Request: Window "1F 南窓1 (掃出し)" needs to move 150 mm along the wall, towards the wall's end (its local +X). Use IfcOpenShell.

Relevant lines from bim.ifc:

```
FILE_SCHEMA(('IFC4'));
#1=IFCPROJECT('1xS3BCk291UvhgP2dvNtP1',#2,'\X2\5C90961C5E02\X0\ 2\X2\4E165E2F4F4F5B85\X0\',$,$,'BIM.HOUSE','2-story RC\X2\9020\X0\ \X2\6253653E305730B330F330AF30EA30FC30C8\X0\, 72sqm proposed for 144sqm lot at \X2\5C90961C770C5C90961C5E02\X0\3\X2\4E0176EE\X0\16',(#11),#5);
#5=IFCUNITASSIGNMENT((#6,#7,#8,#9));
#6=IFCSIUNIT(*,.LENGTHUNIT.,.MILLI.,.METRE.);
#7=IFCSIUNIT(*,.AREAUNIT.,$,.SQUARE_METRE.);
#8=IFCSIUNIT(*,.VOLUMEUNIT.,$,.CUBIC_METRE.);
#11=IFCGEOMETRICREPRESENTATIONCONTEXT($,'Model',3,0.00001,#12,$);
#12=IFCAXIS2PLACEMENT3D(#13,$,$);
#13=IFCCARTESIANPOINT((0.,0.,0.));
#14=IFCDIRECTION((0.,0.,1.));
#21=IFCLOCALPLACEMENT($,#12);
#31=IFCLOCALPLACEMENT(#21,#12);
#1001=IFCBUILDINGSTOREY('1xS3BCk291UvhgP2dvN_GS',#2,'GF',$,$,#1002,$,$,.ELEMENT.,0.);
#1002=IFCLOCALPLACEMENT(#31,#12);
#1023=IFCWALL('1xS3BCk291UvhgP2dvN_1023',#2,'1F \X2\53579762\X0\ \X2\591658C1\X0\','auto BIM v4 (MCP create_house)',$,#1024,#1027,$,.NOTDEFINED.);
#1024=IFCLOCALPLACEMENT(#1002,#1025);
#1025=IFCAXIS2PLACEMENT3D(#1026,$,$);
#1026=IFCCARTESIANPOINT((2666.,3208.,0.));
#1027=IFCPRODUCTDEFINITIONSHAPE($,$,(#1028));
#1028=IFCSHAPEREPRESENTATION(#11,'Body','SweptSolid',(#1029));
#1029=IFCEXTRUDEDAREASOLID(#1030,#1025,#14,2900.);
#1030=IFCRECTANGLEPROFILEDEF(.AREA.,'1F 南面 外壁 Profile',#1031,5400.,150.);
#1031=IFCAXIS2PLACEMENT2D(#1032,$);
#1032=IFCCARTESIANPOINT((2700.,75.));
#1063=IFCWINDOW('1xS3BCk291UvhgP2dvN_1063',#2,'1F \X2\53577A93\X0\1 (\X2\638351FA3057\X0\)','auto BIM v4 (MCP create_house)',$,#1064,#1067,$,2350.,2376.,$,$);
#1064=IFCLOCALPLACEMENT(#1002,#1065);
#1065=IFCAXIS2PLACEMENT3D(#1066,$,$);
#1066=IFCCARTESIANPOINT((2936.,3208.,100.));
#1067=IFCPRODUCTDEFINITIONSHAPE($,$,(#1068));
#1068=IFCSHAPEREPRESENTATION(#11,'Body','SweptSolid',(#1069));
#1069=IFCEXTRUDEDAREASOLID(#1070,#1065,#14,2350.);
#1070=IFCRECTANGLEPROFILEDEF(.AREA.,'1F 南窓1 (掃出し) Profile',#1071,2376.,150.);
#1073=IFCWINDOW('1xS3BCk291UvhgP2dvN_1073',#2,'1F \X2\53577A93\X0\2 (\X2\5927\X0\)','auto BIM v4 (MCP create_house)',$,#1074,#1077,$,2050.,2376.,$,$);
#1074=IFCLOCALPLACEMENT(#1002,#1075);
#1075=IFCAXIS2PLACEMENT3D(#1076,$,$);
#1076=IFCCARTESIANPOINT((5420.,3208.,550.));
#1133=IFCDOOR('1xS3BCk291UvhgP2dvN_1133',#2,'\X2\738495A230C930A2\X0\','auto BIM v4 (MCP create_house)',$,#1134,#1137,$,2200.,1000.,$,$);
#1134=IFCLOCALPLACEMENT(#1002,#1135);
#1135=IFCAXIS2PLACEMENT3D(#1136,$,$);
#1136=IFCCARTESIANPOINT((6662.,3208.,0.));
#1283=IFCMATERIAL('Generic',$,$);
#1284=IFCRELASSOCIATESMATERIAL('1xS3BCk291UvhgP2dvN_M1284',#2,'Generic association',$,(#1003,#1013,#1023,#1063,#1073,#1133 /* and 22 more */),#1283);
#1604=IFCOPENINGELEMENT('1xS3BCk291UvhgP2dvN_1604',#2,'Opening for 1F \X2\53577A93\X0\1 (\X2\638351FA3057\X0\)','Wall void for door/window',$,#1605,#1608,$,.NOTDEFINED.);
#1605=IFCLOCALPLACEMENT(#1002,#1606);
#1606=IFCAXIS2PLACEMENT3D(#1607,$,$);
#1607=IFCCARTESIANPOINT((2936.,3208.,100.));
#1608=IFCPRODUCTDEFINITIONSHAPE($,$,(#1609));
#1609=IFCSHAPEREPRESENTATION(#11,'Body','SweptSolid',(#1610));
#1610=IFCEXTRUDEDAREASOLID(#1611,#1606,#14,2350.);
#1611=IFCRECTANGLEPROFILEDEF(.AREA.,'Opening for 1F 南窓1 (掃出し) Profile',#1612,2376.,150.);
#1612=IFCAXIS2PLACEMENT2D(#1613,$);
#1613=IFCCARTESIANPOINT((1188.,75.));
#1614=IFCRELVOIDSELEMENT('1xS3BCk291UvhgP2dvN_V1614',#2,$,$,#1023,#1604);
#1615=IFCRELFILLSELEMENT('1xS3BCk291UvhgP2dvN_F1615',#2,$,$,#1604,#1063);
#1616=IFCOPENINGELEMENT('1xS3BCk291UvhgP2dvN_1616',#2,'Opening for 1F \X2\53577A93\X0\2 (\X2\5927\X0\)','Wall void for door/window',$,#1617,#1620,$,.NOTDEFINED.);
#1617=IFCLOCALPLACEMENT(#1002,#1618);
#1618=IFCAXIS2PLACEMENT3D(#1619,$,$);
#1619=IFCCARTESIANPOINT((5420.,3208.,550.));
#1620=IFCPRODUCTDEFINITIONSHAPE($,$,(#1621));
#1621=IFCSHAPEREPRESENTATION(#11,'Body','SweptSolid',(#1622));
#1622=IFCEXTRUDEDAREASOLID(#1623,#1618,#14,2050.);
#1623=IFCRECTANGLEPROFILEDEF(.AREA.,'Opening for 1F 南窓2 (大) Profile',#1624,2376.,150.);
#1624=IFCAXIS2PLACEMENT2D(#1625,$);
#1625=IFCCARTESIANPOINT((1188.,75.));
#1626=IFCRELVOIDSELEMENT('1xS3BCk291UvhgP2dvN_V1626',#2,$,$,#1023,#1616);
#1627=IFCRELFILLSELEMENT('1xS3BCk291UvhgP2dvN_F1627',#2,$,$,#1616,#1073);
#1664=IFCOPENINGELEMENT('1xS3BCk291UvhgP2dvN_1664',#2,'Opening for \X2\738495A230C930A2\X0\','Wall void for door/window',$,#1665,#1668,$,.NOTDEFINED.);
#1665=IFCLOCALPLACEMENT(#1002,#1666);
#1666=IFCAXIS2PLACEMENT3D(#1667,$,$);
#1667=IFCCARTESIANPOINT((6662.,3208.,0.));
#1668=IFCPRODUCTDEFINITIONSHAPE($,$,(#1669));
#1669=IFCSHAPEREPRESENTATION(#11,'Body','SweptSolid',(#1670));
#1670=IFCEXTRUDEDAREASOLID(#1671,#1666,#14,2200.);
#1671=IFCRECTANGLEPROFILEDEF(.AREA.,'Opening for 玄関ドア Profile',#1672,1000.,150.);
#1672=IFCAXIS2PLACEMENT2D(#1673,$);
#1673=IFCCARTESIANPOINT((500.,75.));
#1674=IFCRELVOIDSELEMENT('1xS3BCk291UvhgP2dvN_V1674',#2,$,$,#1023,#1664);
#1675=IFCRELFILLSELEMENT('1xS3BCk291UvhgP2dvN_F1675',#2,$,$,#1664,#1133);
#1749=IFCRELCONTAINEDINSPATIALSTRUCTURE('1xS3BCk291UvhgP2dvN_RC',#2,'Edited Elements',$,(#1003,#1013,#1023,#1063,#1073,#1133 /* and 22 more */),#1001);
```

```python
import ifcopenshell
import ifcopenshell.api.geometry
import ifcopenshell.util.placement
import ifcopenshell.util.unit

model = ifcopenshell.open("bim.ifc")
unit_scale = ifcopenshell.util.unit.calculate_unit_scale(model)

window = model.by_guid("1xS3BCk291UvhgP2dvN_1063")
opening = window.FillsVoids[0].RelatingOpeningElement
wall = opening.VoidsElements[0].RelatingBuildingElement

wall_matrix = ifcopenshell.util.placement.get_local_placement(wall.ObjectPlacement)
shift = wall_matrix[:3, 0] * 0.15 / unit_scale
before = ifcopenshell.util.placement.get_local_placement(window.ObjectPlacement)[:3, 3].copy()

# The window is not placed relative to its opening, so move both.
for product in (opening, window):
    matrix = ifcopenshell.util.placement.get_local_placement(product.ObjectPlacement)
    matrix[:3, 3] += shift
    ifcopenshell.api.geometry.edit_object_placement(model, product=product, matrix=matrix, is_si=False)

after = ifcopenshell.util.placement.get_local_placement(window.ObjectPlacement)[:3, 3]
print("window moved by", (after - before).round(3) + 0.0)

model.write("bim_v2.ifc")
```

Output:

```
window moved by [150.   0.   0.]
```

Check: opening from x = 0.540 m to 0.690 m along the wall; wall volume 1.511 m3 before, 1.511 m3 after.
